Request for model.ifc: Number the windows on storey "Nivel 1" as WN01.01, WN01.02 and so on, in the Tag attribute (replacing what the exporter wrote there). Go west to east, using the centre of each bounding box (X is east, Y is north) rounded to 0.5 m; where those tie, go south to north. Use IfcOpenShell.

First a look at what the model holds.

```python
import ifcopenshell
import ifcopenshell.util.element
import ifcopenshell.util.placement

model = ifcopenshell.open("model.ifc")
print(model.schema)
storey = next(s for s in model.by_type("IfcBuildingStorey") if s.Name == "Nivel 1")
windows = [e for e in ifcopenshell.util.element.get_decomposition(storey) if e.is_a("IfcWindow")]
for e in sorted(windows, key=lambda e: e.id()):
    origin = ifcopenshell.util.placement.get_local_placement(e.ObjectPlacement)[:3, 3]
    print(e.id(), e.Tag, e.Name, origin.round(2) + 0.0, sep=" | ")
```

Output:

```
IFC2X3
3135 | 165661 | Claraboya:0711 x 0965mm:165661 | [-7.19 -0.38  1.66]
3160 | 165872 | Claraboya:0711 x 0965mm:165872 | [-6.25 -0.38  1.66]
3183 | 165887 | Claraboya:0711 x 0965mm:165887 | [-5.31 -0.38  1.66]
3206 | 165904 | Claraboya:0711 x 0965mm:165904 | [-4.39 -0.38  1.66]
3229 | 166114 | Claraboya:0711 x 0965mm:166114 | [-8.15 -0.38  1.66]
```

```python
import ifcopenshell
import ifcopenshell.geom
import ifcopenshell.util.element
import ifcopenshell.util.shape

model = ifcopenshell.open("model.ifc")
settings = ifcopenshell.geom.settings()
settings.set("use-world-coords", True)


def centre(element):
    shape = ifcopenshell.geom.create_shape(settings, element)
    return ifcopenshell.util.shape.get_bbox_centroid(shape.geometry)


storey = next(s for s in model.by_type("IfcBuildingStorey") if s.Name == "Nivel 1")
windows = [e for e in ifcopenshell.util.element.get_decomposition(storey) if e.is_a("IfcWindow")]

# Insertion points can sit at a corner or the storey origin, so sort by the geometry (in metres).
centres = {e: centre(e) for e in windows}
windows.sort(key=lambda e: (round(centres[e][0] / 0.5), centres[e][1]))

for i, e in enumerate(windows, start=1):
    number = f"WN01.{i:02d}"
    e.Tag = number
    print(e.id(), number)

model.write("model_rev.ifc")
```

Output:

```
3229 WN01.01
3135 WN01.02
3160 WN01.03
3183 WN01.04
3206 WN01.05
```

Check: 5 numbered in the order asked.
